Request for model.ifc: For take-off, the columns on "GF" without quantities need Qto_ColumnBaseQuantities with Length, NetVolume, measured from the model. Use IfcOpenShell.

First a look at what the model holds.

```python
import ifcopenshell
import ifcopenshell.util.element
import ifcopenshell.util.unit

model = ifcopenshell.open("model.ifc")
print(model.schema)
for unit_type in ("LENGTHUNIT", "AREAUNIT", "VOLUMEUNIT"):
    print(unit_type, ifcopenshell.util.unit.calculate_unit_scale(model, unit_type))
storey = next(s for s in model.by_type("IfcBuildingStorey") if s.Name == "GF")
columns = [e for e in ifcopenshell.util.element.get_decomposition(storey) if e.is_a("IfcColumn")]
for e in sorted(columns, key=lambda e: e.id()):
    print(e.id(), e.is_a(), e.Name, list(ifcopenshell.util.element.get_psets(e, qtos_only=True)), sep=" | ")
```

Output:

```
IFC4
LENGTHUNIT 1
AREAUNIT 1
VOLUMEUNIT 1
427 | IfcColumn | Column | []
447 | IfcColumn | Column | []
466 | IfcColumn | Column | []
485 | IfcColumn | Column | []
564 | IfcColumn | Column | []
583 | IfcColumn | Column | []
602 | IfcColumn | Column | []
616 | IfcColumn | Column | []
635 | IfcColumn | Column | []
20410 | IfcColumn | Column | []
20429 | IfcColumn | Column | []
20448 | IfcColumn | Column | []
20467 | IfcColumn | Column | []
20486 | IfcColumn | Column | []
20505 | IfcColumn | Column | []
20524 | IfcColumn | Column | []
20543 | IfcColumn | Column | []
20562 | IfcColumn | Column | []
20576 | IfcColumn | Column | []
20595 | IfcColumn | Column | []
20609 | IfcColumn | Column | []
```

```python
import ifcopenshell
import ifcopenshell.api.pset
import ifcopenshell.geom
import ifcopenshell.util.element
import ifcopenshell.util.shape
import ifcopenshell.util.unit

model = ifcopenshell.open("model.ifc")
unit_scale = ifcopenshell.util.unit.calculate_unit_scale(model)
volume_scale = ifcopenshell.util.unit.calculate_unit_scale(model, "VOLUMEUNIT")
settings = ifcopenshell.geom.settings()

storey = next(s for s in model.by_type("IfcBuildingStorey") if s.Name == "GF")
columns = [e for e in ifcopenshell.util.element.get_decomposition(storey) if e.is_a("IfcColumn")]

for e in sorted(columns, key=lambda e: e.id()):
    if ifcopenshell.util.element.get_psets(e, qtos_only=True, should_inherit=False):
        continue
    # Geometry comes back in metres, in the element's own axes.
    shape = ifcopenshell.geom.create_shape(settings, e)
    values = {
        "Length": ifcopenshell.util.shape.get_z(shape.geometry) / unit_scale,
        "NetVolume": ifcopenshell.util.shape.get_volume(shape.geometry) / volume_scale,
    }
    qto = ifcopenshell.api.pset.add_qto(model, product=e, name="Qto_ColumnBaseQuantities")
    ifcopenshell.api.pset.edit_qto(model, qto=qto, properties=values)
    print(e.id(), {k: round(v, 3) for k, v in values.items()})

model.write("model-out.ifc")
```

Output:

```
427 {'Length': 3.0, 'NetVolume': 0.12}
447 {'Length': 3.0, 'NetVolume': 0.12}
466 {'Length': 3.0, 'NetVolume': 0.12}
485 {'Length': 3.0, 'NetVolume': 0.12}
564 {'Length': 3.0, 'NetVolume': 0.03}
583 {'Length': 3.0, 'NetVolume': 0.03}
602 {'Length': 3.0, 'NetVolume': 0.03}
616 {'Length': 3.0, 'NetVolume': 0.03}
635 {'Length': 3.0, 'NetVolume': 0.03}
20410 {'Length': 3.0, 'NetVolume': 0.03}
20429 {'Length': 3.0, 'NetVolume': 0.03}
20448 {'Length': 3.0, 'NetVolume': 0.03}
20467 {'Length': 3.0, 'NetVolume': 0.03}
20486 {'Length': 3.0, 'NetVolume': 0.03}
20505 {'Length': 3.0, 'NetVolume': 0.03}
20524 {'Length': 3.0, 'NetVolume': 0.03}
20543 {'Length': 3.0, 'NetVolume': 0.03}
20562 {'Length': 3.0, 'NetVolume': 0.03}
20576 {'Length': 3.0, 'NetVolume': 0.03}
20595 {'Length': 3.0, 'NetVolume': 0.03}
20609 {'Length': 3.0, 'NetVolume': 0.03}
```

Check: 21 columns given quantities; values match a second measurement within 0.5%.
